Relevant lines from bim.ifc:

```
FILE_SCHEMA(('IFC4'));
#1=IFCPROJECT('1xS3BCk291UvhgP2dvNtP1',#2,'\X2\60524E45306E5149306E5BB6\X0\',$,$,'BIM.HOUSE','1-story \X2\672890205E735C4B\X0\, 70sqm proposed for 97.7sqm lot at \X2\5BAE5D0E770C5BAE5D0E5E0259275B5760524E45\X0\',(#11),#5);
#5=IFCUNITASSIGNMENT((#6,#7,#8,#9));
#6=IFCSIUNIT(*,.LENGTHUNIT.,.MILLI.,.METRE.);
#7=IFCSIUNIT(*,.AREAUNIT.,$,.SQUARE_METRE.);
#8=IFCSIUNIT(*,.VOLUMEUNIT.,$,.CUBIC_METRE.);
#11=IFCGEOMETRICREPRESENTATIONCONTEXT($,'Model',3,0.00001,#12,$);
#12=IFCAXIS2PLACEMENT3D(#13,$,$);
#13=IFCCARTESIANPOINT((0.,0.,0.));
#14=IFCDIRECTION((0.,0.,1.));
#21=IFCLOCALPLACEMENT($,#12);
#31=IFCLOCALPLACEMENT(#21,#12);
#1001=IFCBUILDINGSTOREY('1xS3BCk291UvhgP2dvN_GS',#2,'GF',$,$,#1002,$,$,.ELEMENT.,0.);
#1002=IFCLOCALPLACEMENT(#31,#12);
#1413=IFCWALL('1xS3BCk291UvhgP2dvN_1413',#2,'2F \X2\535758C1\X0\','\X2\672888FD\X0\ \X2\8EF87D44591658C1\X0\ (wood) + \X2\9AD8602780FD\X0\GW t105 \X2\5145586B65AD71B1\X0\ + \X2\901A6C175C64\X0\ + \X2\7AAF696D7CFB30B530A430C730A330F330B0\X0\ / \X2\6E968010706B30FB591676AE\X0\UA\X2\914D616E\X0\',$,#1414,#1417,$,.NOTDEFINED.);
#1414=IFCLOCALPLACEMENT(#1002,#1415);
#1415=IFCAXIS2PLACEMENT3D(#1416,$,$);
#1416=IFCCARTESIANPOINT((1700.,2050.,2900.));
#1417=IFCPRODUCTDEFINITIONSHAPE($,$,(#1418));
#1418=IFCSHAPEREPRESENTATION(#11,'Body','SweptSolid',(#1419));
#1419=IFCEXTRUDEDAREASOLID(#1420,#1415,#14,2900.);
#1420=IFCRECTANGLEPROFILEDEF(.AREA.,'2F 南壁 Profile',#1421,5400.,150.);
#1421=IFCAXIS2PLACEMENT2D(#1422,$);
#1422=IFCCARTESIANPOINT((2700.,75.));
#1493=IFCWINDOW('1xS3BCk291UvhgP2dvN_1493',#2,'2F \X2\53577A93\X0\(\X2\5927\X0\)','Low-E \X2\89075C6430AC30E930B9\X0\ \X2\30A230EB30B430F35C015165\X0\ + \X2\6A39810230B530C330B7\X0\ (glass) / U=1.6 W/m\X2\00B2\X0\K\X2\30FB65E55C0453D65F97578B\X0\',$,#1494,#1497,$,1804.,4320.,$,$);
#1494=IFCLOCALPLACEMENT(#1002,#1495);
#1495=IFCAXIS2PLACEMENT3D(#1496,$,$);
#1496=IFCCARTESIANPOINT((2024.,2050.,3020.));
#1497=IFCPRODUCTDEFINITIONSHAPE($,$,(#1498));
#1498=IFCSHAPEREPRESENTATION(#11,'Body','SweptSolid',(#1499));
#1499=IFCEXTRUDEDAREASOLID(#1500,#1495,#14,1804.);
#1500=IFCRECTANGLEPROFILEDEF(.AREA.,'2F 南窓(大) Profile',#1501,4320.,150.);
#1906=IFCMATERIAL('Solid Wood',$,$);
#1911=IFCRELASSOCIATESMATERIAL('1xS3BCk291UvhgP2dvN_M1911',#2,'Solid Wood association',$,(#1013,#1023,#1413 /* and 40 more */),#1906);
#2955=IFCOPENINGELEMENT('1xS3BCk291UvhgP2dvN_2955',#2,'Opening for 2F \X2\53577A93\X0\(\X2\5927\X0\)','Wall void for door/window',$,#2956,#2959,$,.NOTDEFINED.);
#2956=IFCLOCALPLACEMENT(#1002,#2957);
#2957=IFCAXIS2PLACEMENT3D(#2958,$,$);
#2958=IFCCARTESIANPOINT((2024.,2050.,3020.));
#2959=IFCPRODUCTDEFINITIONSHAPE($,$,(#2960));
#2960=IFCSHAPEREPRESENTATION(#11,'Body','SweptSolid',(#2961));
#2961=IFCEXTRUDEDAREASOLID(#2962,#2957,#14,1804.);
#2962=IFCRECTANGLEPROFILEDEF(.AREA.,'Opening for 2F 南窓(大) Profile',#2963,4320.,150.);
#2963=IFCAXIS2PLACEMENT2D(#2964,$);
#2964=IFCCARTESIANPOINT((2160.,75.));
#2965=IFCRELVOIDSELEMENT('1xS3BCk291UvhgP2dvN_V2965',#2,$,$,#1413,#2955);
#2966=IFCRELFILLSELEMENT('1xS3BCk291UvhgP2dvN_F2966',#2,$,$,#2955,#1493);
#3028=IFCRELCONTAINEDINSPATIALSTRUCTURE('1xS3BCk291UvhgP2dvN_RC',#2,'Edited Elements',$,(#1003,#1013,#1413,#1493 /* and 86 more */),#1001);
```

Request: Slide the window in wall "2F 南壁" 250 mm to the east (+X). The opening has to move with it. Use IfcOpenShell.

```python
import ifcopenshell
import ifcopenshell.api.geometry
import ifcopenshell.util.placement
import ifcopenshell.util.unit

model = ifcopenshell.open("bim.ifc")
unit_scale = ifcopenshell.util.unit.calculate_unit_scale(model)

window = model.by_guid("1xS3BCk291UvhgP2dvN_1493")
opening = window.FillsVoids[0].RelatingOpeningElement
wall = opening.VoidsElements[0].RelatingBuildingElement

wall_matrix = ifcopenshell.util.placement.get_local_placement(wall.ObjectPlacement)
shift = wall_matrix[:3, 0] * 0.25 / unit_scale
before = ifcopenshell.util.placement.get_local_placement(window.ObjectPlacement)[:3, 3].copy()

# The window is not placed relative to its opening, so move both.
for product in (opening, window):
    matrix = ifcopenshell.util.placement.get_local_placement(product.ObjectPlacement)
    matrix[:3, 3] += shift
    ifcopenshell.api.geometry.edit_object_placement(model, product=product, matrix=matrix, is_si=False)

after = ifcopenshell.util.placement.get_local_placement(window.ObjectPlacement)[:3, 3]
print("window moved by", (after - before).round(3) + 0.0)

model.write("bim_v2.ifc")
```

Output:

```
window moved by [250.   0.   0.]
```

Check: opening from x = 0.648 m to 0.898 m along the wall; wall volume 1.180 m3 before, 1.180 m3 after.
